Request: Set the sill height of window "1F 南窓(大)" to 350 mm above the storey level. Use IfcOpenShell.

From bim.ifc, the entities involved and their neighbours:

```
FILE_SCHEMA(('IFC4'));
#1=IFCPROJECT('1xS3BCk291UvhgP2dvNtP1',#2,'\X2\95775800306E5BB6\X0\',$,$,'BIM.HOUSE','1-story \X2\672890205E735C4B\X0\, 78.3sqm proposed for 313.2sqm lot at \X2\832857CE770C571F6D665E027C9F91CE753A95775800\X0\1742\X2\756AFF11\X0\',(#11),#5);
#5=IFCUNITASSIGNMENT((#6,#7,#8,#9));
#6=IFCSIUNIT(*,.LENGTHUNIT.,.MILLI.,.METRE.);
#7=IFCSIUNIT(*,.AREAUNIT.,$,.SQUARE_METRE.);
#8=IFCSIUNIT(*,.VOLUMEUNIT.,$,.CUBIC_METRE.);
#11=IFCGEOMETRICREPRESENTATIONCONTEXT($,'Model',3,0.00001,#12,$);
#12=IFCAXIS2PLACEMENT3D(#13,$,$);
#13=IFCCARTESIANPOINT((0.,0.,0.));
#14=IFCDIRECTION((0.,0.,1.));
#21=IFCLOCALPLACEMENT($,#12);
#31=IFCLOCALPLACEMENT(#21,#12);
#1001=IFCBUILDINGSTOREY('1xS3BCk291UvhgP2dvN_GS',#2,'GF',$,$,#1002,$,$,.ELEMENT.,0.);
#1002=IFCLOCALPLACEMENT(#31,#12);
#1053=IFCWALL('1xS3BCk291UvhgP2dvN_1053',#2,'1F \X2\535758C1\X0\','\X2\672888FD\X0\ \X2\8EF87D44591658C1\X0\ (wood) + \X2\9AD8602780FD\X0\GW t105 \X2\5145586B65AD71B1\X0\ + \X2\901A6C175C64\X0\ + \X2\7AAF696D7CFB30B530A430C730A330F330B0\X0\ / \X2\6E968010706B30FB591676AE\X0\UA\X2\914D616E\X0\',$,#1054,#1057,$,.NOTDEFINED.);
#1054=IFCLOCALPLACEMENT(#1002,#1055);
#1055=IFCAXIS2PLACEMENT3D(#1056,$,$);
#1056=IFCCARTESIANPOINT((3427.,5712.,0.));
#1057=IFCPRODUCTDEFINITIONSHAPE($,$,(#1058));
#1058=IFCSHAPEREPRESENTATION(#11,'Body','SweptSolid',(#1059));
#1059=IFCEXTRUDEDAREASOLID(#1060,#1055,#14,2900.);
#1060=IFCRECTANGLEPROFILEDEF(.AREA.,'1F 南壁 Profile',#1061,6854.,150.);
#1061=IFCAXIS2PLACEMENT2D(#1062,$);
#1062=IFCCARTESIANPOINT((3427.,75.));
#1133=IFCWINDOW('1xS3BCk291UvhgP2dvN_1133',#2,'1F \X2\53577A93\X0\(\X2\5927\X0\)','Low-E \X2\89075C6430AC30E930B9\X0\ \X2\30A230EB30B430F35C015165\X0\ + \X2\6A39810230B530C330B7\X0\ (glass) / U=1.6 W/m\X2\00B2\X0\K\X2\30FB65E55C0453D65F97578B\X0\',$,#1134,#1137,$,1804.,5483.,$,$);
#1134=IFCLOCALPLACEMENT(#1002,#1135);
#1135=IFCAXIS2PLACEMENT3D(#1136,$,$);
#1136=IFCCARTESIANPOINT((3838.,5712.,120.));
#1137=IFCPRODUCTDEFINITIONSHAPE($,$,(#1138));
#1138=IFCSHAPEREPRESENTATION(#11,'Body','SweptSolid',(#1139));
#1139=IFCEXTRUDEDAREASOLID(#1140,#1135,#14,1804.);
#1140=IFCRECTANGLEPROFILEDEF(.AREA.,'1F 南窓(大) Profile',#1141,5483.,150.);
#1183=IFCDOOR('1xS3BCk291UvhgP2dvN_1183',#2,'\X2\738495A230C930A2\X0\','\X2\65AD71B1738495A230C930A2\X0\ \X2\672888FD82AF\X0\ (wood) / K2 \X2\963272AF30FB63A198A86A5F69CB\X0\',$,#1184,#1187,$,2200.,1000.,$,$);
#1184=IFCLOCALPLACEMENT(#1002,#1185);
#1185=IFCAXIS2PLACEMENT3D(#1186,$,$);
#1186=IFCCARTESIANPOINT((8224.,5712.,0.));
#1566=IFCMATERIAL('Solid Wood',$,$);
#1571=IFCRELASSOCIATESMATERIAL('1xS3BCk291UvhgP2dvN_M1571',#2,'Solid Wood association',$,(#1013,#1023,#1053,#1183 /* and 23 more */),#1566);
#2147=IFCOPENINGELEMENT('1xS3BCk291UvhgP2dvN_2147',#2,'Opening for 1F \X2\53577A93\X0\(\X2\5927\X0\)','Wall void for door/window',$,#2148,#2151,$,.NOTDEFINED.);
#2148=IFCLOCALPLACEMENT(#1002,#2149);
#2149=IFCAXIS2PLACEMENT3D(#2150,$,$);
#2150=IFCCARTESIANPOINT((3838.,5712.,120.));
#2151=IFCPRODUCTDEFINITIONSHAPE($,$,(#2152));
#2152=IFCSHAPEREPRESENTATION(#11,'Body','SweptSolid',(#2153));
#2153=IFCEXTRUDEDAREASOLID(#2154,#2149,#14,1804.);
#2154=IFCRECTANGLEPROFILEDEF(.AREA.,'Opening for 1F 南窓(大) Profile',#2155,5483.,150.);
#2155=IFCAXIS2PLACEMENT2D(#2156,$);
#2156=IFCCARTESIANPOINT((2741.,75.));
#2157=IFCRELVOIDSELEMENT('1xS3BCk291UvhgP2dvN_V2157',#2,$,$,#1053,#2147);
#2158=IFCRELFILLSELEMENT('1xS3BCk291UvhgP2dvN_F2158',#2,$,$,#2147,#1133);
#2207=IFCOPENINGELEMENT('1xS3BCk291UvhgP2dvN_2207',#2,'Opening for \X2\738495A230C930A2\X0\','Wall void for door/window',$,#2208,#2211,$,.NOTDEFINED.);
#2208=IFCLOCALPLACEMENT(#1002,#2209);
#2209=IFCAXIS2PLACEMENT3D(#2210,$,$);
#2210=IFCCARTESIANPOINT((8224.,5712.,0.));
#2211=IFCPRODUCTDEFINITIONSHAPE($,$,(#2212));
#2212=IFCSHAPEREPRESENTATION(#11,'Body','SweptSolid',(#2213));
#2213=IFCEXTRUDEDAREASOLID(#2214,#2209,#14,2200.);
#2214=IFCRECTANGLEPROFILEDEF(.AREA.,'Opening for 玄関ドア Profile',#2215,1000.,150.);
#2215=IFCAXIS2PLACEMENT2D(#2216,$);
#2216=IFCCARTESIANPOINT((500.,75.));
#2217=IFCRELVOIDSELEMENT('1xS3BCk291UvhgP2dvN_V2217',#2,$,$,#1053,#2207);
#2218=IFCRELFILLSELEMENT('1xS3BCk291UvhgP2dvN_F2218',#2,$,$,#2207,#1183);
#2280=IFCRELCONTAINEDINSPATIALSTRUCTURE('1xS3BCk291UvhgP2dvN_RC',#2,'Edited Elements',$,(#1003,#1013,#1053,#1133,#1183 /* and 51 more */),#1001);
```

```python
import numpy as np
import ifcopenshell
import ifcopenshell.api.geometry
import ifcopenshell.geom
import ifcopenshell.util.element
import ifcopenshell.util.placement
import ifcopenshell.util.shape
import ifcopenshell.util.unit

model = ifcopenshell.open("bim.ifc")
unit_scale = ifcopenshell.util.unit.calculate_unit_scale(model)

window = model.by_guid("1xS3BCk291UvhgP2dvN_1133")
opening = window.FillsVoids[0].RelatingOpeningElement
storey = ifcopenshell.util.element.get_container(window, ifc_class="IfcBuildingStorey")
level = ifcopenshell.util.placement.get_local_placement(storey.ObjectPlacement)[2, 3]

# The opening's origin need not be at the sill, so measure its lowest point.
shape = ifcopenshell.geom.create_shape(ifcopenshell.geom.settings(), opening)
bottom = ifcopenshell.util.shape.get_shape_bottom_elevation(shape, shape.geometry) / unit_scale
dz = level + 0.35 / unit_scale - bottom

shift = np.array([0.0, 0.0, dz])
# The window is not placed relative to its opening, so move both.
for product in (opening, window):
    matrix = ifcopenshell.util.placement.get_local_placement(product.ObjectPlacement)
    matrix[:3, 3] += shift
    ifcopenshell.api.geometry.edit_object_placement(model, product=product, matrix=matrix, is_si=False)

print(f"moved by {dz * unit_scale:+.3f} m")

model.write("bim-out.ifc")
```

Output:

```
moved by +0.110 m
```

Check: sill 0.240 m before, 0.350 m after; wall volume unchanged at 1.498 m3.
